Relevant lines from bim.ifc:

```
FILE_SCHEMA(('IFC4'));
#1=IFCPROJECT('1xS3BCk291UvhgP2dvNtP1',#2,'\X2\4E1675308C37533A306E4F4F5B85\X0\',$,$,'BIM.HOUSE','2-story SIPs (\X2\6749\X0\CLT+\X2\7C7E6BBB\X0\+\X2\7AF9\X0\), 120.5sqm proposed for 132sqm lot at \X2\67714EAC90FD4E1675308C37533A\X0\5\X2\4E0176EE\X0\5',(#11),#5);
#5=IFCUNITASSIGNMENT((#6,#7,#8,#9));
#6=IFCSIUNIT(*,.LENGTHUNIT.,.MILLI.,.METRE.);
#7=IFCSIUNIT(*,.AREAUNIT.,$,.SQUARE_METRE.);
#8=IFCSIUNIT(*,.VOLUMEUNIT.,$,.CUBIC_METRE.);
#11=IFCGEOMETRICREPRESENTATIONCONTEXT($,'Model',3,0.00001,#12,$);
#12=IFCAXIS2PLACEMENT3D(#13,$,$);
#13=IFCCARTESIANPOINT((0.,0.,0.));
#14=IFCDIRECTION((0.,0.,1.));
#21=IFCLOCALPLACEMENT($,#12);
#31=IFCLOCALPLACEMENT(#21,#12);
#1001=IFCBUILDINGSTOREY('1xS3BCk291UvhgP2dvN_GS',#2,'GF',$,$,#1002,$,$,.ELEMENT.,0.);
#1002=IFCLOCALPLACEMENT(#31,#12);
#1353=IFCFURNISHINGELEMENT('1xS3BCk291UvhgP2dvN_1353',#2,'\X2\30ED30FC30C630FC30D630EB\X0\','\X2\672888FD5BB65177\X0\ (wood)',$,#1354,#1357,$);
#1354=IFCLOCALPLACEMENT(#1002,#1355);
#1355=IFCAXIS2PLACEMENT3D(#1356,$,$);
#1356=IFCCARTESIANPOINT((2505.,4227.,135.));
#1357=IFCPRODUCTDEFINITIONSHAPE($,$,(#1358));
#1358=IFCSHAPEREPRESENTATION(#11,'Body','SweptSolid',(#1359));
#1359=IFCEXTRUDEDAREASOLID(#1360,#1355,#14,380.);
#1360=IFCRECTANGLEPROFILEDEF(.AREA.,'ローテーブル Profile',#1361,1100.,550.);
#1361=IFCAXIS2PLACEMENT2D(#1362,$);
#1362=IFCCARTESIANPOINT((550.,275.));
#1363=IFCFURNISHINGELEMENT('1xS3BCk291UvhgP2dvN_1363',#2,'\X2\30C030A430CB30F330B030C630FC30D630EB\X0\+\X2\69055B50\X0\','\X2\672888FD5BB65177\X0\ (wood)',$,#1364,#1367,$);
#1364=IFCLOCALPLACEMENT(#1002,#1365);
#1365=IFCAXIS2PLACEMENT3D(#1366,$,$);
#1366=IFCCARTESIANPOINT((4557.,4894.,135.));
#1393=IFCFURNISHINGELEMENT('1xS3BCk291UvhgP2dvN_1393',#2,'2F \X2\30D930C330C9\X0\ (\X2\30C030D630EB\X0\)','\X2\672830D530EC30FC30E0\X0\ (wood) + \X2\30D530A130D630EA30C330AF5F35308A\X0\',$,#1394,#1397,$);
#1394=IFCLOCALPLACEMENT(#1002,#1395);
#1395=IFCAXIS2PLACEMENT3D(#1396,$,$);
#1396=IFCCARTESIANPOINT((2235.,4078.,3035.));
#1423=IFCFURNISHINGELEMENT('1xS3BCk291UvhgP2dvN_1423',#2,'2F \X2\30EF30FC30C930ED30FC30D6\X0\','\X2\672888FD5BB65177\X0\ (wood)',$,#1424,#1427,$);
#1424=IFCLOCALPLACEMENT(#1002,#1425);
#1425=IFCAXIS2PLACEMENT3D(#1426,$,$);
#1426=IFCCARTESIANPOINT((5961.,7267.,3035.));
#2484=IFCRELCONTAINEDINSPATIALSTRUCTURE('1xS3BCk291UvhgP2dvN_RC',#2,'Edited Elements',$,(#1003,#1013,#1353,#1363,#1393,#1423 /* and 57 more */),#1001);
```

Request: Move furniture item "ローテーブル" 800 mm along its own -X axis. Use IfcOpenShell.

```python
import ifcopenshell
import ifcopenshell.api.geometry
import ifcopenshell.util.placement
import ifcopenshell.util.unit

model = ifcopenshell.open("bim.ifc")
unit_scale = ifcopenshell.util.unit.calculate_unit_scale(model)

item = model.by_guid("1xS3BCk291UvhgP2dvN_1353")
matrix = ifcopenshell.util.placement.get_local_placement(item.ObjectPlacement)
matrix[:3, 3] -= matrix[:3, 0] * 0.8 / unit_scale
ifcopenshell.api.geometry.edit_object_placement(model, product=item, matrix=matrix, is_si=False)

print(ifcopenshell.util.placement.get_local_placement(item.ObjectPlacement).round(3) + 0.0)

model.write("bim_updated.ifc")
```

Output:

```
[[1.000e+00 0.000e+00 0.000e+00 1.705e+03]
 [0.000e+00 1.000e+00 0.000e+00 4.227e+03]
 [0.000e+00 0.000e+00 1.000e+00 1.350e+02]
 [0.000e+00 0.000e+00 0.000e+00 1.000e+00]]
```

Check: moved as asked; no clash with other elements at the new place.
